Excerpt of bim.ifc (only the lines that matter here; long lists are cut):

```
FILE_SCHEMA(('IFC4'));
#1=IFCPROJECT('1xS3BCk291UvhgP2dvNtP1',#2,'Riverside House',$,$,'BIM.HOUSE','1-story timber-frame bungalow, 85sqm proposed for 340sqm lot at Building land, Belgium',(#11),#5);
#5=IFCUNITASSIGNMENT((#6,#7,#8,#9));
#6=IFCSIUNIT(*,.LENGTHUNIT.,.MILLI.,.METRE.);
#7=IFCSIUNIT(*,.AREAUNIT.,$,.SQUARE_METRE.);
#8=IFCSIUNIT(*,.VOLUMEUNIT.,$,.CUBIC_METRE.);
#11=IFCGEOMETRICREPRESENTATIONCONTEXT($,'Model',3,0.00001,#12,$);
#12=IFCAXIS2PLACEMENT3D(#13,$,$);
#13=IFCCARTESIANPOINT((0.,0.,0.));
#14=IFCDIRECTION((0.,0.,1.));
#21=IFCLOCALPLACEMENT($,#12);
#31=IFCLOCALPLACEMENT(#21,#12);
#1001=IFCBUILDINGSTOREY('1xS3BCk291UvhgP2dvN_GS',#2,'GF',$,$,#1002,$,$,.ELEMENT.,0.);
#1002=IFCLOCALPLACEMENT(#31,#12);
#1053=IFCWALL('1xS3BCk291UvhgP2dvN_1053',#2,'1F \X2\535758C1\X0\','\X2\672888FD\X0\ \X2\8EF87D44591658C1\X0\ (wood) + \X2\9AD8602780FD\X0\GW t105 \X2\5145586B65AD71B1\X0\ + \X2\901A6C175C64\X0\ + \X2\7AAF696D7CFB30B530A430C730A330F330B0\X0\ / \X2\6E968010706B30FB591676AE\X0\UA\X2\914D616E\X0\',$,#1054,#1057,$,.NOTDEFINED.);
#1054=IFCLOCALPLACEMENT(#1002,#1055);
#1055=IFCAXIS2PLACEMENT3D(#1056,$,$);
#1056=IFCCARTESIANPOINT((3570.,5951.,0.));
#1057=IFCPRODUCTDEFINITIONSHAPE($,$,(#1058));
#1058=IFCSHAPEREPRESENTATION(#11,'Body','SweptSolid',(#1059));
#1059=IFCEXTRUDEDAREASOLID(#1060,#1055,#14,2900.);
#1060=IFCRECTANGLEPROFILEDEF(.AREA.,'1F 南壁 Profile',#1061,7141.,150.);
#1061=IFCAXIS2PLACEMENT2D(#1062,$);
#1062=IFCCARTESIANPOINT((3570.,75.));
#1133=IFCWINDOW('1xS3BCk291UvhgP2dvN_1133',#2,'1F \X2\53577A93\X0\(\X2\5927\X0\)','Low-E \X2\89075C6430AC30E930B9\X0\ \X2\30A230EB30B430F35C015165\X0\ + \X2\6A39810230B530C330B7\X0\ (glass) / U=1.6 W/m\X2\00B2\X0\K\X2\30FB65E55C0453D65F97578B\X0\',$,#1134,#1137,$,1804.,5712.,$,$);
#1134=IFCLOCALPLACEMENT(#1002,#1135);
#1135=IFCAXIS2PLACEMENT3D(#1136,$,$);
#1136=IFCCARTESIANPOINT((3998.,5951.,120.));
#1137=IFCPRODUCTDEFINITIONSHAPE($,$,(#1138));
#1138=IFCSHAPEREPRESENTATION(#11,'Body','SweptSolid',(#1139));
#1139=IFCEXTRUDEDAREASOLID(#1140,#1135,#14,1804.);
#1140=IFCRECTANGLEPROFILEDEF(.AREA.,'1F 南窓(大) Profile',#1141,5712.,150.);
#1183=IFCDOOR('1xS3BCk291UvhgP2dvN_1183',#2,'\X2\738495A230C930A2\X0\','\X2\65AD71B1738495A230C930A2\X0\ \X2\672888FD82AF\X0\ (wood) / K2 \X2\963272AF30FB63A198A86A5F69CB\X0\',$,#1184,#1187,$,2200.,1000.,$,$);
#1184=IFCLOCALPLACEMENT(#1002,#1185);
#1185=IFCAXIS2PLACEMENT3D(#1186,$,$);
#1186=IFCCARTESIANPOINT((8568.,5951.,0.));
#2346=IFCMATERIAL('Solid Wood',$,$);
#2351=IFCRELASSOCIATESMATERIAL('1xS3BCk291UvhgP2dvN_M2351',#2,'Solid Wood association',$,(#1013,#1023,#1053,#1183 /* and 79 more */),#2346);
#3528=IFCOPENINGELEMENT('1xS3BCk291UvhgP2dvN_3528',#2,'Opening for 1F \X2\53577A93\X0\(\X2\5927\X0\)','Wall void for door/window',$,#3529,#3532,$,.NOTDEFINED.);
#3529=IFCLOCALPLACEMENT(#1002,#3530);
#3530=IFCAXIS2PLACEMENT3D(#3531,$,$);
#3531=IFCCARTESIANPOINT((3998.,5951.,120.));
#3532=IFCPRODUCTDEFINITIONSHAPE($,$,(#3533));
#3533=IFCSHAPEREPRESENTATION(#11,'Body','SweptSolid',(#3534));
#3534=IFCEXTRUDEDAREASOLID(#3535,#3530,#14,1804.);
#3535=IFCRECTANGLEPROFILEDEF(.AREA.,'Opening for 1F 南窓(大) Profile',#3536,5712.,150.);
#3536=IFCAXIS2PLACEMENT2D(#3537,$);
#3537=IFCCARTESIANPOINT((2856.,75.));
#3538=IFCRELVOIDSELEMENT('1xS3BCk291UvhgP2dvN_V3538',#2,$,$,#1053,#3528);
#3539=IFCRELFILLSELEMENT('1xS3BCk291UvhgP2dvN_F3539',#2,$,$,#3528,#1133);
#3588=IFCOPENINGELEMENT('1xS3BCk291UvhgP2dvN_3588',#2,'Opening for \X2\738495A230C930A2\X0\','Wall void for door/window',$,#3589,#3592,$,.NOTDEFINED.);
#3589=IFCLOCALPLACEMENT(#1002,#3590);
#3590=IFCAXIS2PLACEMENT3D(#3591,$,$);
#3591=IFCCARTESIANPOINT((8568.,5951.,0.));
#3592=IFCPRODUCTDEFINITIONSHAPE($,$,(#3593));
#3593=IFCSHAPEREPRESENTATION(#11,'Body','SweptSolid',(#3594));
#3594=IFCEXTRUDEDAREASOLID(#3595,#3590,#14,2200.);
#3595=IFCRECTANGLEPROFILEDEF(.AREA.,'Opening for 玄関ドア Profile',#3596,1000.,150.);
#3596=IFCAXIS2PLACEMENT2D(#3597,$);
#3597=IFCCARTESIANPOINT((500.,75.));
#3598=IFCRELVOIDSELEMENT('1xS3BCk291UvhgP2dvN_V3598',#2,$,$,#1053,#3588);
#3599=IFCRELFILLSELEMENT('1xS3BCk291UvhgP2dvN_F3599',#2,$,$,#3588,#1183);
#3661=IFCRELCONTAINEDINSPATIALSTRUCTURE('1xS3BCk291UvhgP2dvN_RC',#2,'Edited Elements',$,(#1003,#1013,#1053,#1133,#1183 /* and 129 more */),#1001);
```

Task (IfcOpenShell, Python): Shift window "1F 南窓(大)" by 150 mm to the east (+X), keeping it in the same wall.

```python
import ifcopenshell
import ifcopenshell.api.geometry
import ifcopenshell.util.placement

model = ifcopenshell.open("bim.ifc")

window = model.by_id(1133)
opening = window.FillsVoids[0].RelatingOpeningElement
wall = opening.VoidsElements[0].RelatingBuildingElement

wall_matrix = ifcopenshell.util.placement.get_local_placement(wall.ObjectPlacement)
shift = wall_matrix[:3, 0] * 150.0
before = ifcopenshell.util.placement.get_local_placement(window.ObjectPlacement)[:3, 3].copy()

# The window is not placed relative to its opening, so move both.
for product in (opening, window):
    matrix = ifcopenshell.util.placement.get_local_placement(product.ObjectPlacement)
    matrix[:3, 3] += shift
    ifcopenshell.api.geometry.edit_object_placement(model, product=product, matrix=matrix, is_si=False)

after = ifcopenshell.util.placement.get_local_placement(window.ObjectPlacement)[:3, 3]
print("window moved by", (after - before).round(3) + 0.0)

model.write("bim_rev.ifc")
```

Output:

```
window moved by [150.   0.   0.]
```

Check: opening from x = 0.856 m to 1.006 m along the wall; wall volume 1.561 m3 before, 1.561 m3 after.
